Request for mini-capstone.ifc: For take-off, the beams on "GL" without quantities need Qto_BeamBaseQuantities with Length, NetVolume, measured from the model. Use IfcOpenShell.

First a look at what the model holds.

```python
import ifcopenshell
import ifcopenshell.util.element
import ifcopenshell.util.unit

model = ifcopenshell.open("mini-capstone.ifc")
print(model.schema)
for unit_type in ("LENGTHUNIT", "AREAUNIT", "VOLUMEUNIT"):
    print(unit_type, ifcopenshell.util.unit.calculate_unit_scale(model, unit_type))
storey = next(s for s in model.by_type("IfcBuildingStorey") if s.Name == "GL")
beams = [e for e in ifcopenshell.util.element.get_decomposition(storey) if e.is_a("IfcBeam")]
for e in sorted(beams, key=lambda e: e.id()):
    print(e.id(), e.is_a(), e.Name, list(ifcopenshell.util.element.get_psets(e, qtos_only=True)), sep=" | ")
```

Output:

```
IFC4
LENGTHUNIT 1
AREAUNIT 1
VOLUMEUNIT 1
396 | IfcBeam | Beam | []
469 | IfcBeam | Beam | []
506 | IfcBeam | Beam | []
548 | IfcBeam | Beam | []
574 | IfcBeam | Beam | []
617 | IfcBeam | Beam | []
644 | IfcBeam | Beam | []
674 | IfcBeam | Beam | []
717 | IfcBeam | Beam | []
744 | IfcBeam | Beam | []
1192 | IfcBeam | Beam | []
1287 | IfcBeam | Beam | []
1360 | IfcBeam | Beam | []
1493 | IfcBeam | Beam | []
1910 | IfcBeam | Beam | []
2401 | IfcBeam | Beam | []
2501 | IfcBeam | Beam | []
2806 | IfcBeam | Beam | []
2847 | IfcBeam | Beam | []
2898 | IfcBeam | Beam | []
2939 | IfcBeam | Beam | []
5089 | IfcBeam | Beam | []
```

```python
import ifcopenshell
import ifcopenshell.api.pset
import ifcopenshell.geom
import ifcopenshell.util.element
import ifcopenshell.util.shape
import ifcopenshell.util.unit

model = ifcopenshell.open("mini-capstone.ifc")
unit_scale = ifcopenshell.util.unit.calculate_unit_scale(model)
volume_scale = ifcopenshell.util.unit.calculate_unit_scale(model, "VOLUMEUNIT")
settings = ifcopenshell.geom.settings()

storey = next(s for s in model.by_type("IfcBuildingStorey") if s.Name == "GL")
beams = [e for e in ifcopenshell.util.element.get_decomposition(storey) if e.is_a("IfcBeam")]

for e in sorted(beams, key=lambda e: e.id()):
    if ifcopenshell.util.element.get_psets(e, qtos_only=True, should_inherit=False):
        continue
    # Geometry comes back in metres, in the element's own axes.
    shape = ifcopenshell.geom.create_shape(settings, e)
    values = {
        "Length": ifcopenshell.util.shape.get_max_xyz(shape.geometry) / unit_scale,
        "NetVolume": ifcopenshell.util.shape.get_volume(shape.geometry) / volume_scale,
    }
    qto = ifcopenshell.api.pset.add_qto(model, product=e, name="Qto_BeamBaseQuantities")
    ifcopenshell.api.pset.edit_qto(model, qto=qto, properties=values)
    print(e.id(), {k: round(v, 3) for k, v in values.items()})

model.write("mini-capstone_edited.ifc")
```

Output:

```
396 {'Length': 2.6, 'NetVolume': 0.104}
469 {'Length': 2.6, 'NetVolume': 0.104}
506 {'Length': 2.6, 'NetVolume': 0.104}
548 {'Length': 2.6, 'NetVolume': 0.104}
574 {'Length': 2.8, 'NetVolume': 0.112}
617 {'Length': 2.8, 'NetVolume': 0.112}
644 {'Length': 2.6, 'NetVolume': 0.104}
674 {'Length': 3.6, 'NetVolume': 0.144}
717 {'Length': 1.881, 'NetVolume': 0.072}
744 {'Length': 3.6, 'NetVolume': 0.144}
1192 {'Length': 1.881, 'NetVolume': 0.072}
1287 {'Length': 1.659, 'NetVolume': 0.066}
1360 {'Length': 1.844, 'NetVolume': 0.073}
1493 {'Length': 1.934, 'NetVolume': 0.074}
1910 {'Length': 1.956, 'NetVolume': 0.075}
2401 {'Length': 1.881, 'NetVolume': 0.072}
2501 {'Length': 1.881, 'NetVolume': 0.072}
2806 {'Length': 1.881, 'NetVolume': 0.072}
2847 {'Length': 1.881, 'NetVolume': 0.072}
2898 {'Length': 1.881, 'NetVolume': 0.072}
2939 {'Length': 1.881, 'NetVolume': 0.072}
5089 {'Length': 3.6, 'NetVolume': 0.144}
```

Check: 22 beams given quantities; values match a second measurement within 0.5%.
